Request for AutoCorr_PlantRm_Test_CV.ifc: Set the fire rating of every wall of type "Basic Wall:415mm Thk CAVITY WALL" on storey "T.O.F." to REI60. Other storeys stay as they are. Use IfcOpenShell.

First a look at what the model holds.

```python
import ifcopenshell
import ifcopenshell.util.element

model = ifcopenshell.open("AutoCorr_PlantRm_Test_CV.ifc")
print(model.schema)
storey = next(s for s in model.by_type("IfcBuildingStorey") if s.Name == "T.O.F.")
walls = [e for e in ifcopenshell.util.element.get_decomposition(storey) if e.is_a("IfcWall")]
seen = {}
for e in walls:
    element_type = ifcopenshell.util.element.get_type(e)
    key = (element_type.Name if element_type != e and element_type else None, ifcopenshell.util.element.get_pset(e, "Pset_WallCommon", "FireRating"))
    seen[key] = seen.get(key, 0) + 1
for (name, value), count in sorted(seen.items(), key=str):
    print(count, "x", name, "|", value)
```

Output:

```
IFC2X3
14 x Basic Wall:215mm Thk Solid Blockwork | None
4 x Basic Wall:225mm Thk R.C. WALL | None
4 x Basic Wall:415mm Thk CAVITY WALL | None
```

```python
import ifcopenshell
import ifcopenshell.api.pset
import ifcopenshell.util.element

model = ifcopenshell.open("AutoCorr_PlantRm_Test_CV.ifc")

storey = next(s for s in model.by_type("IfcBuildingStorey") if s.Name == "T.O.F.")
walls = [e for e in ifcopenshell.util.element.get_decomposition(storey) if e.is_a("IfcWall")]

count = 0
for e in walls:
    element_type = ifcopenshell.util.element.get_type(e)
    if element_type in (None, e) or element_type.Name != "Basic Wall:415mm Thk CAVITY WALL":
        continue
    # add_pset returns the element's existing set when there is one.
    pset = ifcopenshell.api.pset.add_pset(model, product=e, name="Pset_WallCommon")
    ifcopenshell.api.pset.edit_pset(model, pset=pset, properties={"FireRating": "REI60"})
    count += 1

print(count, "walls updated")

model.write("AutoCorr_PlantRm_Test_CV_rev.ifc")
```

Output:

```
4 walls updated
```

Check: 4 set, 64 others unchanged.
